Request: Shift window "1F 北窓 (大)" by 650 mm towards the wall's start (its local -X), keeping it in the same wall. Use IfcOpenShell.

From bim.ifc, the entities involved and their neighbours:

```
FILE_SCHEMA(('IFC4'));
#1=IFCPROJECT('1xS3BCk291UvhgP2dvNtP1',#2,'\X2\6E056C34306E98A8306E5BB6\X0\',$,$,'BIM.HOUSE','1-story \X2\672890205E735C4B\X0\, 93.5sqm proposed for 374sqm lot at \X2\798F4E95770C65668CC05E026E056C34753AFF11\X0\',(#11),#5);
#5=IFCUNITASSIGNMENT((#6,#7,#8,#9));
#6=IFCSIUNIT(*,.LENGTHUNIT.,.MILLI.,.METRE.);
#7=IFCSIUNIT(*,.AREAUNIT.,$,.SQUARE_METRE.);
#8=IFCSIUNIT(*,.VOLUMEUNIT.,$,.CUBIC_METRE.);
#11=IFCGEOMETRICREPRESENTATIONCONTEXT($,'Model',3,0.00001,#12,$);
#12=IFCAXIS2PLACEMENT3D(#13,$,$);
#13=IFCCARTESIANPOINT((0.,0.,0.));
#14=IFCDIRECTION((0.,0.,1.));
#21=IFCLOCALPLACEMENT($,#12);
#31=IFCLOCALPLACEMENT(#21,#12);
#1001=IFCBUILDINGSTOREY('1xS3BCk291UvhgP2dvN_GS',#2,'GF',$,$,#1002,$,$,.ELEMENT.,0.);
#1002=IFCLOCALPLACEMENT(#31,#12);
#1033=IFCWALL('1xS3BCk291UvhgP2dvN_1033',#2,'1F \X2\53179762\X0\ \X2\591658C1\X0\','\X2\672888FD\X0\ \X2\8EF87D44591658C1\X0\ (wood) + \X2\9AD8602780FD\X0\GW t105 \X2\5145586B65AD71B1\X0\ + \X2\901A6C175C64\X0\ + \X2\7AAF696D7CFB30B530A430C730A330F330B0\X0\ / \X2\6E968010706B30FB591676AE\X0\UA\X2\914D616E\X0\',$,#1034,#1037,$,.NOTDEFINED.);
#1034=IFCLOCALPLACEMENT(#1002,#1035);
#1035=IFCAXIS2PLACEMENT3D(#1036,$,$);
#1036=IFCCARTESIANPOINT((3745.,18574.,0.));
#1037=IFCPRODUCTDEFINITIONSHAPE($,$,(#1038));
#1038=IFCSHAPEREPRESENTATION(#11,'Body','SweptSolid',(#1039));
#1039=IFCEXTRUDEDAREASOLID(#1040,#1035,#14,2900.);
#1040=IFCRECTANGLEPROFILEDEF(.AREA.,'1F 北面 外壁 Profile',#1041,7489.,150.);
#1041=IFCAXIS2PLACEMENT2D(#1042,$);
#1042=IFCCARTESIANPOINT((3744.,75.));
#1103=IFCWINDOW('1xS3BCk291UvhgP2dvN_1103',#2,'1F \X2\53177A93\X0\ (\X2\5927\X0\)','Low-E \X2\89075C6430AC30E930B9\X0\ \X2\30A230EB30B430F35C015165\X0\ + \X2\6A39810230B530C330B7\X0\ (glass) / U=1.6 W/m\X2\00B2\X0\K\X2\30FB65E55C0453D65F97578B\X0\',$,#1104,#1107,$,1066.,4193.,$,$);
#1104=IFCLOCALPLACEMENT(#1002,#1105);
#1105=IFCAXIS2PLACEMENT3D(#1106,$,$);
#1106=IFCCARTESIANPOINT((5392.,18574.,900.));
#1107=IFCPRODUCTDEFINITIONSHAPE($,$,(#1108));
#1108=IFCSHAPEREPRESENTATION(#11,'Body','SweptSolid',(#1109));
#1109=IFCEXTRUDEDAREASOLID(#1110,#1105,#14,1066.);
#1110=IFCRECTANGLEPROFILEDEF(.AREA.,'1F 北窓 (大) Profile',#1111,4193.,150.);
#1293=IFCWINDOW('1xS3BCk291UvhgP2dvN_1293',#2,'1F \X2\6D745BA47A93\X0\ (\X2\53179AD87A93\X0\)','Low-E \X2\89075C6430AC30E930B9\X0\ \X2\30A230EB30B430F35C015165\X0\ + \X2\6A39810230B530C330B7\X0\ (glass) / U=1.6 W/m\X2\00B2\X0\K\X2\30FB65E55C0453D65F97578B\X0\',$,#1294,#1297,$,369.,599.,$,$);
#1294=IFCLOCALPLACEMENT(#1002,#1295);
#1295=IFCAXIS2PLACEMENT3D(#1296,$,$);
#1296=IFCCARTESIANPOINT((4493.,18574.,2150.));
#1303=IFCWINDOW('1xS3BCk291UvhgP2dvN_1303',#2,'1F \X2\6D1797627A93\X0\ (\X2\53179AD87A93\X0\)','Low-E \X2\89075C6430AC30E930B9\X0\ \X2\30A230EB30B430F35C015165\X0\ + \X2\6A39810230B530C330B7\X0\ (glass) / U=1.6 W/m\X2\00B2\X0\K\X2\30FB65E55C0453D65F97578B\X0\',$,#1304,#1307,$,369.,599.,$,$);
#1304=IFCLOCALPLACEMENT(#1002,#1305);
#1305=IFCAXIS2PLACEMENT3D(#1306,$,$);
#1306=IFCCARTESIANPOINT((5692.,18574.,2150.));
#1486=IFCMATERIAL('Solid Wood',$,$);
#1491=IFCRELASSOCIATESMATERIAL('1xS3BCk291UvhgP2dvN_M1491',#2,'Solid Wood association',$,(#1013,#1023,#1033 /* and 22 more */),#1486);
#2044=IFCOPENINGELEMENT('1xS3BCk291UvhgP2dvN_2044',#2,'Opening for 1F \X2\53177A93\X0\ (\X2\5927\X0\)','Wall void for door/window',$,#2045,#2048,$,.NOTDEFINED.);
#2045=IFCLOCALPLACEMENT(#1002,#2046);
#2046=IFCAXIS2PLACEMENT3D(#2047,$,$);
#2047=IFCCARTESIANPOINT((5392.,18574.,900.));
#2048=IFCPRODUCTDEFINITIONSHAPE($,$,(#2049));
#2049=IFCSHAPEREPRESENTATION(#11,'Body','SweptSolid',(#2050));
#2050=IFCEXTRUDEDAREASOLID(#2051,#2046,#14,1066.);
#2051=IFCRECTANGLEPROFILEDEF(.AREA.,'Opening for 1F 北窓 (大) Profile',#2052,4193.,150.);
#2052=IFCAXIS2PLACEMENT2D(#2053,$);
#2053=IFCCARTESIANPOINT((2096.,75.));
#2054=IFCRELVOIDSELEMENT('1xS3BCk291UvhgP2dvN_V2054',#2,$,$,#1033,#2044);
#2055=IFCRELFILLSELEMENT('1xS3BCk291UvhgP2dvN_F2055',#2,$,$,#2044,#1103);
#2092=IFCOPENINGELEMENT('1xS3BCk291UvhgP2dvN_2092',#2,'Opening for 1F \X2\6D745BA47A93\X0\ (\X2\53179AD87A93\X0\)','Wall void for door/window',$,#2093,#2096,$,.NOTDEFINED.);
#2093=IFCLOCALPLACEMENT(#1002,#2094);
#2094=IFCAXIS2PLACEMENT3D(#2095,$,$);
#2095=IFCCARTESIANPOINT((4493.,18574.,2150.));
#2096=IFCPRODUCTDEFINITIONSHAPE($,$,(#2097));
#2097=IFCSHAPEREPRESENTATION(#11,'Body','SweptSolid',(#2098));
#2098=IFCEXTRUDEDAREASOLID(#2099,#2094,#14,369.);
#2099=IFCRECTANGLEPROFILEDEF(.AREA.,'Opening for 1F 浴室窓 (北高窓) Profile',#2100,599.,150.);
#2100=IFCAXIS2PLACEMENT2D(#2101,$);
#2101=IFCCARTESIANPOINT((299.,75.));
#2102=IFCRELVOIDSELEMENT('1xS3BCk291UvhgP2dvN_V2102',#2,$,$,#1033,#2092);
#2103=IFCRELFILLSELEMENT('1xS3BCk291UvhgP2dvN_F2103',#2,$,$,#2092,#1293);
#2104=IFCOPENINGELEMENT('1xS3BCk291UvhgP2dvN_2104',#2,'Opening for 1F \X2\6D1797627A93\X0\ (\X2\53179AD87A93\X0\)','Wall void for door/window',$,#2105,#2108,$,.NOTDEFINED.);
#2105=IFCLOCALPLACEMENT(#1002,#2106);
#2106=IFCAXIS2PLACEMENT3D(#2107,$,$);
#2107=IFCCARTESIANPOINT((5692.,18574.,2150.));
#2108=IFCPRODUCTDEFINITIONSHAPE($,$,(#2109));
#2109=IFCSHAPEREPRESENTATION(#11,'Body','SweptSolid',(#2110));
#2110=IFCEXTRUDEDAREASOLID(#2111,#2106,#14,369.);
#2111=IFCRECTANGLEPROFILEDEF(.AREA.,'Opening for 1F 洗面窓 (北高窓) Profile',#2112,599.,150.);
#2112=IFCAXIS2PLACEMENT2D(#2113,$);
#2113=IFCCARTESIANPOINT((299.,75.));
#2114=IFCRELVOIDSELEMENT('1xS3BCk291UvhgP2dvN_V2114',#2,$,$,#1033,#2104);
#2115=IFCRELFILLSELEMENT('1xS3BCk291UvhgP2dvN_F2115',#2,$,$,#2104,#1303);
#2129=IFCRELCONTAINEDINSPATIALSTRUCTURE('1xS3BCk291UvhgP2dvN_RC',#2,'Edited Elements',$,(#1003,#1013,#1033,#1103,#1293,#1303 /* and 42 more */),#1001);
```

```python
import ifcopenshell
import ifcopenshell.api.geometry
import ifcopenshell.util.placement
import ifcopenshell.util.unit

model = ifcopenshell.open("bim.ifc")
unit_scale = ifcopenshell.util.unit.calculate_unit_scale(model)

window = model.by_guid("1xS3BCk291UvhgP2dvN_1103")
opening = window.FillsVoids[0].RelatingOpeningElement
wall = opening.VoidsElements[0].RelatingBuildingElement

wall_matrix = ifcopenshell.util.placement.get_local_placement(wall.ObjectPlacement)
shift = wall_matrix[:3, 0] * -0.65 / unit_scale
before = ifcopenshell.util.placement.get_local_placement(window.ObjectPlacement)[:3, 3].copy()

# The window is not placed relative to its opening, so move both.
for product in (opening, window):
    matrix = ifcopenshell.util.placement.get_local_placement(product.ObjectPlacement)
    matrix[:3, 3] += shift
    ifcopenshell.api.geometry.edit_object_placement(model, product=product, matrix=matrix, is_si=False)

after = ifcopenshell.util.placement.get_local_placement(window.ObjectPlacement)[:3, 3]
print("window moved by", (after - before).round(3) + 0.0)

model.write("bim_v2.ifc")
```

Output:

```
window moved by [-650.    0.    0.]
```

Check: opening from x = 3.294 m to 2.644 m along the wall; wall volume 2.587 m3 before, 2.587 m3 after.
